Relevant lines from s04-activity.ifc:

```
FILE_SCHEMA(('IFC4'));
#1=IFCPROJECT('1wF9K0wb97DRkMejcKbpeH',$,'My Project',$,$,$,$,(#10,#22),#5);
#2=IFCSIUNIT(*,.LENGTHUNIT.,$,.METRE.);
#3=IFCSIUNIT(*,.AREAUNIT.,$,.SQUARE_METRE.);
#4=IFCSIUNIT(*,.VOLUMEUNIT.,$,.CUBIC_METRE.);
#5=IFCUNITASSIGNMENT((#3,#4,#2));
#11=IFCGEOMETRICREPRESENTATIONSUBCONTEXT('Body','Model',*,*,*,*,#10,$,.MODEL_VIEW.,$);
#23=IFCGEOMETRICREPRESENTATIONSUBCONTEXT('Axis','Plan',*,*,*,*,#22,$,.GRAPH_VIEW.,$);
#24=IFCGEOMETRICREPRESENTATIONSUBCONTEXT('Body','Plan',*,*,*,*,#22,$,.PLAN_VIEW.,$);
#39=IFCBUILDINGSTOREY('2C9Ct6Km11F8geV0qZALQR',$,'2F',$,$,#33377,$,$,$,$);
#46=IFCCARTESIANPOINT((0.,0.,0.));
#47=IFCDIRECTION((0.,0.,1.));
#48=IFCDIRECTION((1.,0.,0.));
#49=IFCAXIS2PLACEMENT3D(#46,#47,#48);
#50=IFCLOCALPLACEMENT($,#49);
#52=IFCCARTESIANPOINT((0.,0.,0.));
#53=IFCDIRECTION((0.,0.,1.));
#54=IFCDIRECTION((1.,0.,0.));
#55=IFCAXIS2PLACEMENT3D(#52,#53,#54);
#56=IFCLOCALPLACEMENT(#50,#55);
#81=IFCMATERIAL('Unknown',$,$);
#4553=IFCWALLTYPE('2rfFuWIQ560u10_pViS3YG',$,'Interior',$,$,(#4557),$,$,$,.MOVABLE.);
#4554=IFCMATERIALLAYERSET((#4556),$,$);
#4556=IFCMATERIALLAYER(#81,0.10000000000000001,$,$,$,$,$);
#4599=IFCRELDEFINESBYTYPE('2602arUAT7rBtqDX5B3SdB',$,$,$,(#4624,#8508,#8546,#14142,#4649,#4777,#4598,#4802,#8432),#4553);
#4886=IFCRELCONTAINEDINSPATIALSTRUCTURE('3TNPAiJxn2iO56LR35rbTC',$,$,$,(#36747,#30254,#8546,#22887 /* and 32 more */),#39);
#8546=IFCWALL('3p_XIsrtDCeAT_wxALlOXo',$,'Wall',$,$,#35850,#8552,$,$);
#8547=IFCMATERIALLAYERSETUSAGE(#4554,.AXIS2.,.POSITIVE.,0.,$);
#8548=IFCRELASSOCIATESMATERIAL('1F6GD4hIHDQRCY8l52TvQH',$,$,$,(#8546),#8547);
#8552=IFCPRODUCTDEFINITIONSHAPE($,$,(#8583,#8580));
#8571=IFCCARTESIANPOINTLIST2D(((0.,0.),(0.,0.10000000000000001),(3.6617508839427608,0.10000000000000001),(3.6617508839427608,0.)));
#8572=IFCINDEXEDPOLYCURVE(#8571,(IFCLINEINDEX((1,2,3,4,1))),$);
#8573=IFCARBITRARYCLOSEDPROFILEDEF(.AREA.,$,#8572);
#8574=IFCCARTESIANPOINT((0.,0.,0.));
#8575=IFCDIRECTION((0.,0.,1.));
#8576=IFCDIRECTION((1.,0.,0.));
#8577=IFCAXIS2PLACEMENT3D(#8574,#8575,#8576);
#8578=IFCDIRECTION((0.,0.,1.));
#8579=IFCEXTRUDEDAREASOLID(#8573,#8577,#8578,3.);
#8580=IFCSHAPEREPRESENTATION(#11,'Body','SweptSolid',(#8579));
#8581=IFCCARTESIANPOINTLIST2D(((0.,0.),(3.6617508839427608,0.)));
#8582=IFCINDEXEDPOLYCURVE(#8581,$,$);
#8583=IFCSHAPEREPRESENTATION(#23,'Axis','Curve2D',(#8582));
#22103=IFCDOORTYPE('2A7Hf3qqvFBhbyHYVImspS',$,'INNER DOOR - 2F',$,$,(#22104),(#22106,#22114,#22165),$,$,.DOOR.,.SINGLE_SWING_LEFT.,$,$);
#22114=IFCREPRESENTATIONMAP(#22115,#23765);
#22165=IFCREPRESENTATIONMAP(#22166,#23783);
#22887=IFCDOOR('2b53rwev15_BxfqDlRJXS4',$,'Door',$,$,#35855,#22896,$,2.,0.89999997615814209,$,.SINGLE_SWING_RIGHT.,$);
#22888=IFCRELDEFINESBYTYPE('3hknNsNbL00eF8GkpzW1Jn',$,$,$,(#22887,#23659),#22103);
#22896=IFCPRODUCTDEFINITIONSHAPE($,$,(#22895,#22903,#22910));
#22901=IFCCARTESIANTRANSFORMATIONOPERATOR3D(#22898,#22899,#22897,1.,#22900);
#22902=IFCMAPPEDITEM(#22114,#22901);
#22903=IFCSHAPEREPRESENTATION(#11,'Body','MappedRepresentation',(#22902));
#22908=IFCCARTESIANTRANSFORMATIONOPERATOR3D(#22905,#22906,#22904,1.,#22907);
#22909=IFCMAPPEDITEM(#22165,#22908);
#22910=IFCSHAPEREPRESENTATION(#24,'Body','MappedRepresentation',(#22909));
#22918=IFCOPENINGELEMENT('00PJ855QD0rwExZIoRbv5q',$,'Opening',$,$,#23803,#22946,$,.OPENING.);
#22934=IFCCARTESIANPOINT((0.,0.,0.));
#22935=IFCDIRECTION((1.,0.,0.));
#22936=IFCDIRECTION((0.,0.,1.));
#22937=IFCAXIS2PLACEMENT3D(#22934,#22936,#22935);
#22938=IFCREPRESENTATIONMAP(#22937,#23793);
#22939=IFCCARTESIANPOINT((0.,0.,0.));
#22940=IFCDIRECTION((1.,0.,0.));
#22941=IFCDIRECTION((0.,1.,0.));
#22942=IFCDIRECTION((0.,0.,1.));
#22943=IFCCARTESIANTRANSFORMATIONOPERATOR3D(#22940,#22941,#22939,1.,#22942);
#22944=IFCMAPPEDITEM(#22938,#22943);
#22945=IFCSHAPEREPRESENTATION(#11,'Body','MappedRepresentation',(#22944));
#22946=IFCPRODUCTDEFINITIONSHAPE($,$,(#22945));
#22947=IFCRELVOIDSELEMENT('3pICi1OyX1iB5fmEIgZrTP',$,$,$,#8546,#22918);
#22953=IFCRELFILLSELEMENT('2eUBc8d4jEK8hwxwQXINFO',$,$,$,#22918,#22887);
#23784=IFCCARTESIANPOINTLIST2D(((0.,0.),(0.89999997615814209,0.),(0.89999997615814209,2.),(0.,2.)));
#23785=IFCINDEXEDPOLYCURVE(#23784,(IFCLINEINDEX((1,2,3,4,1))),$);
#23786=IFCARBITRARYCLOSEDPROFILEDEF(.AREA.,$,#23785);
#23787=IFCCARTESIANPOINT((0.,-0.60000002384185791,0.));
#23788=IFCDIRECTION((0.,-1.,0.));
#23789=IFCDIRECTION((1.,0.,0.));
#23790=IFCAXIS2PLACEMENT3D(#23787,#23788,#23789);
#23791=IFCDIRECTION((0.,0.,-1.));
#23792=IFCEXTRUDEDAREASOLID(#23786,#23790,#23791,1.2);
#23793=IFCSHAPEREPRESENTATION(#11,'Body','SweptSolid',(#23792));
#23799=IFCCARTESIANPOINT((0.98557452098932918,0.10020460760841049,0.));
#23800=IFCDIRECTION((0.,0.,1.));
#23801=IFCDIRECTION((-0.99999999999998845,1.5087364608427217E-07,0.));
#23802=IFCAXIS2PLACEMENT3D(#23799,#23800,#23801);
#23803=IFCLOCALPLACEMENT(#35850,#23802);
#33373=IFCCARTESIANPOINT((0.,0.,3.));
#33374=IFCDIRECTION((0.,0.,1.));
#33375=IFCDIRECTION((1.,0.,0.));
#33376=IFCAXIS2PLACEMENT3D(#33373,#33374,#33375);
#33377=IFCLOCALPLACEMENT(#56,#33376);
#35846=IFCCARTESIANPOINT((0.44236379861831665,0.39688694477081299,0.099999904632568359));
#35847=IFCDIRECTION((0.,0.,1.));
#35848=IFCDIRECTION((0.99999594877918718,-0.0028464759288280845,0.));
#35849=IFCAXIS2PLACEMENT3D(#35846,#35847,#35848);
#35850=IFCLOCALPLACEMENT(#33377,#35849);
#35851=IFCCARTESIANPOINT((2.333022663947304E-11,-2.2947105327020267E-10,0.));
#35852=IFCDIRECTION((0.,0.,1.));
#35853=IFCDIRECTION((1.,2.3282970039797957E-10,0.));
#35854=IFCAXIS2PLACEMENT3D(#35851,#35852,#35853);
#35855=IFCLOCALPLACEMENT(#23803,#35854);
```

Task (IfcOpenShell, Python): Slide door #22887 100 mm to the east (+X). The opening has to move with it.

```python
import ifcopenshell
import ifcopenshell.api.geometry
import ifcopenshell.util.placement
import ifcopenshell.util.unit

model = ifcopenshell.open("s04-activity.ifc")
unit_scale = ifcopenshell.util.unit.calculate_unit_scale(model)

door = model.by_guid("2b53rwev15_BxfqDlRJXS4")
opening = door.FillsVoids[0].RelatingOpeningElement
wall = opening.VoidsElements[0].RelatingBuildingElement

wall_matrix = ifcopenshell.util.placement.get_local_placement(wall.ObjectPlacement)
shift = wall_matrix[:3, 0] * 0.1 / unit_scale
before = ifcopenshell.util.placement.get_local_placement(door.ObjectPlacement)[:3, 3].copy()

# The door is placed relative to its opening, so it follows when the opening moves.
matrix = ifcopenshell.util.placement.get_local_placement(opening.ObjectPlacement)
matrix[:3, 3] += shift
ifcopenshell.api.geometry.edit_object_placement(
    model, product=opening, matrix=matrix, is_si=False, should_transform_children=True
)

after = ifcopenshell.util.placement.get_local_placement(door.ObjectPlacement)[:3, 3]
print("door moved by", (after - before).round(3) + 0.0)

model.write("s04-activity_edited.ifc")
```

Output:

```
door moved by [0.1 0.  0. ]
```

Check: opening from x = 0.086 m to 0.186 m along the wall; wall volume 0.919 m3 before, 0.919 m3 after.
